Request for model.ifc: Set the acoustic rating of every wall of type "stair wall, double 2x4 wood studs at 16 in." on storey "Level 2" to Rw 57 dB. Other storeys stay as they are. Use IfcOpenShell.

First a look at what the model holds.

```python
import ifcopenshell
import ifcopenshell.util.element

model = ifcopenshell.open("model.ifc")
print(model.schema)
storey = next(s for s in model.by_type("IfcBuildingStorey") if s.Name == "Level 2")
walls = [e for e in ifcopenshell.util.element.get_decomposition(storey) if e.is_a("IfcWall")]
seen = {}
for e in walls:
    element_type = ifcopenshell.util.element.get_type(e)
    key = (element_type.Name if element_type != e and element_type else None, ifcopenshell.util.element.get_pset(e, "Pset_WallCommon", "AcousticRating"))
    seen[key] = seen.get(key, 0) + 1
for (name, value), count in sorted(seen.items(), key=str):
    print(count, "x", name, "|", value)
```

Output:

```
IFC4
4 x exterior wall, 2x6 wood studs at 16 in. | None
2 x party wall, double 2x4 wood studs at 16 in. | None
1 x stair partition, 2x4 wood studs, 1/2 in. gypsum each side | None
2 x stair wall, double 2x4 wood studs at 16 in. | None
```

```python
import ifcopenshell
import ifcopenshell.api.pset
import ifcopenshell.util.element

model = ifcopenshell.open("model.ifc")

storey = next(s for s in model.by_type("IfcBuildingStorey") if s.Name == "Level 2")
walls = [e for e in ifcopenshell.util.element.get_decomposition(storey) if e.is_a("IfcWall")]

count = 0
for e in walls:
    element_type = ifcopenshell.util.element.get_type(e)
    if element_type in (None, e) or element_type.Name != "stair wall, double 2x4 wood studs at 16 in.":
        continue
    # add_pset returns the element's existing set when there is one.
    pset = ifcopenshell.api.pset.add_pset(model, product=e, name="Pset_WallCommon")
    ifcopenshell.api.pset.edit_pset(model, pset=pset, properties={"AcousticRating": "Rw 57 dB"})
    count += 1

print(count, "walls updated")

model.write("model_v2.ifc")
```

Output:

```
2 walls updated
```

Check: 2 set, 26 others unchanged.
